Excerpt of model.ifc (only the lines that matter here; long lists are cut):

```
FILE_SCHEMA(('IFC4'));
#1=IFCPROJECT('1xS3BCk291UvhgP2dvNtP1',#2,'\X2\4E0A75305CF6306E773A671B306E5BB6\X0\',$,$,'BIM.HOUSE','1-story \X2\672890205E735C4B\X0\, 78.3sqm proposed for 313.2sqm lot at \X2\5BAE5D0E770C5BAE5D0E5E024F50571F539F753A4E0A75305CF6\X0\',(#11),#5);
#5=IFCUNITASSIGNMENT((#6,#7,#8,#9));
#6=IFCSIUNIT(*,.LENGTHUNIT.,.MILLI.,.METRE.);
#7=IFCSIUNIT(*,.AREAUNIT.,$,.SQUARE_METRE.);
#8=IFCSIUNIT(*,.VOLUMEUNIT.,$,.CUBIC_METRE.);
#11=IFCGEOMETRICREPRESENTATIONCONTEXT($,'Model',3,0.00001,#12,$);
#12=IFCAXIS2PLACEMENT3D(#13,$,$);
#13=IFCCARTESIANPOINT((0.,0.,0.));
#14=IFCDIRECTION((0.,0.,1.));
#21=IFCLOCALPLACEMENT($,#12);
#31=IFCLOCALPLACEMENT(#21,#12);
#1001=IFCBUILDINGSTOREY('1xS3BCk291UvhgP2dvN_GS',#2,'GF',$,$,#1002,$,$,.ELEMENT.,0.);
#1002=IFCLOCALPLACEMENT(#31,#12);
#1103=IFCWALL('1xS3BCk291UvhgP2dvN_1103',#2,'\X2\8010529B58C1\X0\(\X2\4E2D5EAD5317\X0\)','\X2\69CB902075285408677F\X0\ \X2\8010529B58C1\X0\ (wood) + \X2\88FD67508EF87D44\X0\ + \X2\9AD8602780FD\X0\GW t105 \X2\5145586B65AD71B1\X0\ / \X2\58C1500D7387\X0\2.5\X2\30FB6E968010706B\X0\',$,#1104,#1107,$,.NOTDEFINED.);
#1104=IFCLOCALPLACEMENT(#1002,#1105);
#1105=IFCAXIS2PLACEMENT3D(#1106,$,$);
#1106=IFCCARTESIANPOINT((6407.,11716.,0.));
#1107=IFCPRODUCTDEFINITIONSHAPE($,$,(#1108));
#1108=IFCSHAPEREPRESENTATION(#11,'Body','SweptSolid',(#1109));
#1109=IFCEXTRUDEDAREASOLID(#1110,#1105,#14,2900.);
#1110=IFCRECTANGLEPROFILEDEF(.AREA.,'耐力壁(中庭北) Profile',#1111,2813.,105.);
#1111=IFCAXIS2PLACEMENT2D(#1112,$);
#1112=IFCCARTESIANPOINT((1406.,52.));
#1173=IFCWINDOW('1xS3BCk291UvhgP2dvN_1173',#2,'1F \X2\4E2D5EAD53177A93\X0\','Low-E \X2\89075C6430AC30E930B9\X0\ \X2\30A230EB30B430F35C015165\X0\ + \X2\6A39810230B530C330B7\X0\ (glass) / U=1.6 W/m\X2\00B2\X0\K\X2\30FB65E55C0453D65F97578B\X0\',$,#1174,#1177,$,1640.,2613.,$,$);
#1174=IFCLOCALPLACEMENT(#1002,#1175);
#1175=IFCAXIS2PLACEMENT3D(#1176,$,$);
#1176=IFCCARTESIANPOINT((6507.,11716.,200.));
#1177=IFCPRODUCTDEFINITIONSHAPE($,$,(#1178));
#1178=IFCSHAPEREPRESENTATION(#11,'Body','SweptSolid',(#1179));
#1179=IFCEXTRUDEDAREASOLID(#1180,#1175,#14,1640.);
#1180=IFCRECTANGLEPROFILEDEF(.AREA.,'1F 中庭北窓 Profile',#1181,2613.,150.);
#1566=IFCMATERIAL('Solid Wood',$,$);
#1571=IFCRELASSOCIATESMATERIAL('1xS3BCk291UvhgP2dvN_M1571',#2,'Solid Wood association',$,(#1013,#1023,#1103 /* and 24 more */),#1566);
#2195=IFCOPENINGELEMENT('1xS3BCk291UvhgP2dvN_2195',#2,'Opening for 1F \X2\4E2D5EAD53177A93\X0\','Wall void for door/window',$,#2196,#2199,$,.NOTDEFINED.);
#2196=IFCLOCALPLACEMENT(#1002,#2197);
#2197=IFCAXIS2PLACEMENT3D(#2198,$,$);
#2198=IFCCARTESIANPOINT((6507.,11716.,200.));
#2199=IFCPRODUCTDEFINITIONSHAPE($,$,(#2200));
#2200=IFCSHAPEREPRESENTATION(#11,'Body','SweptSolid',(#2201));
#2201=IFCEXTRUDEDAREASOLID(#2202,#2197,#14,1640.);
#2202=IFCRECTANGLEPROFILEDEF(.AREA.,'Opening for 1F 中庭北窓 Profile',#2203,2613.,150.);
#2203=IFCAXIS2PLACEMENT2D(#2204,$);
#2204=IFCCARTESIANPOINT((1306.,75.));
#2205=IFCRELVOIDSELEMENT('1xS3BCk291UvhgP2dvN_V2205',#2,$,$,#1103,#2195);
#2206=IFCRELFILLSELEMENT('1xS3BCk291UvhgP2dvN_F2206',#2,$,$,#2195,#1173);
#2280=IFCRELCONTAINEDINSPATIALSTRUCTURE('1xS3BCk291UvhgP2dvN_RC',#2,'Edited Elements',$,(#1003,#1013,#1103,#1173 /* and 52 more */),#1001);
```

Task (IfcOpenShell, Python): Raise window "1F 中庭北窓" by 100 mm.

```python
import numpy as np
import ifcopenshell
import ifcopenshell.api.geometry
import ifcopenshell.util.placement
import ifcopenshell.util.unit

model = ifcopenshell.open("model.ifc")
unit_scale = ifcopenshell.util.unit.calculate_unit_scale(model)

window = model.by_guid("1xS3BCk291UvhgP2dvN_1173")
opening = window.FillsVoids[0].RelatingOpeningElement
dz = 100.0

shift = np.array([0.0, 0.0, dz])
# The window is not placed relative to its opening, so move both.
for product in (opening, window):
    matrix = ifcopenshell.util.placement.get_local_placement(product.ObjectPlacement)
    matrix[:3, 3] += shift
    ifcopenshell.api.geometry.edit_object_placement(model, product=product, matrix=matrix, is_si=False)

print(f"moved by {dz * unit_scale:+.3f} m")

model.write("model_edited.ifc")
```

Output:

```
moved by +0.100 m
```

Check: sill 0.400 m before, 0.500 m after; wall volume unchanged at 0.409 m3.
